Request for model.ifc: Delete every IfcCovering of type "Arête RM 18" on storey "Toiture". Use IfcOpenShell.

First a look at what the model holds.

```python
import ifcopenshell
import ifcopenshell.util.element

model = ifcopenshell.open("model.ifc")
print(model.schema)
storey = next(s for s in model.by_type("IfcBuildingStorey") if s.Name == "Toiture")
coverings = [e for e in ifcopenshell.util.element.get_decomposition(storey) if e.is_a("IfcCovering")]
seen = {}
for e in coverings:
    element_type = ifcopenshell.util.element.get_type(e)
    name = element_type.Name if element_type not in (None, e) else None
    seen[name] = seen.get(name, 0) + 1
for name, count in sorted(seen.items(), key=str):
    print(count, "x", name)
```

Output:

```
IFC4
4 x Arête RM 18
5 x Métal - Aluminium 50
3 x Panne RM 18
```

```python
import ifcopenshell
import ifcopenshell.api.root
import ifcopenshell.util.element

model = ifcopenshell.open("model.ifc")

storey = next(s for s in model.by_type("IfcBuildingStorey") if s.Name == "Toiture")
coverings = [e for e in ifcopenshell.util.element.get_decomposition(storey) if e.is_a("IfcCovering")]
targets = [e for e in coverings if (t := ifcopenshell.util.element.get_type(e)) not in (None, e) and t.Name == "Arête RM 18"]

for e in targets:
    ifcopenshell.api.root.remove_product(model, product=e)
print(len(targets), "removed")

model.write("model_updated.ifc")
```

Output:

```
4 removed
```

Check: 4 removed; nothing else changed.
